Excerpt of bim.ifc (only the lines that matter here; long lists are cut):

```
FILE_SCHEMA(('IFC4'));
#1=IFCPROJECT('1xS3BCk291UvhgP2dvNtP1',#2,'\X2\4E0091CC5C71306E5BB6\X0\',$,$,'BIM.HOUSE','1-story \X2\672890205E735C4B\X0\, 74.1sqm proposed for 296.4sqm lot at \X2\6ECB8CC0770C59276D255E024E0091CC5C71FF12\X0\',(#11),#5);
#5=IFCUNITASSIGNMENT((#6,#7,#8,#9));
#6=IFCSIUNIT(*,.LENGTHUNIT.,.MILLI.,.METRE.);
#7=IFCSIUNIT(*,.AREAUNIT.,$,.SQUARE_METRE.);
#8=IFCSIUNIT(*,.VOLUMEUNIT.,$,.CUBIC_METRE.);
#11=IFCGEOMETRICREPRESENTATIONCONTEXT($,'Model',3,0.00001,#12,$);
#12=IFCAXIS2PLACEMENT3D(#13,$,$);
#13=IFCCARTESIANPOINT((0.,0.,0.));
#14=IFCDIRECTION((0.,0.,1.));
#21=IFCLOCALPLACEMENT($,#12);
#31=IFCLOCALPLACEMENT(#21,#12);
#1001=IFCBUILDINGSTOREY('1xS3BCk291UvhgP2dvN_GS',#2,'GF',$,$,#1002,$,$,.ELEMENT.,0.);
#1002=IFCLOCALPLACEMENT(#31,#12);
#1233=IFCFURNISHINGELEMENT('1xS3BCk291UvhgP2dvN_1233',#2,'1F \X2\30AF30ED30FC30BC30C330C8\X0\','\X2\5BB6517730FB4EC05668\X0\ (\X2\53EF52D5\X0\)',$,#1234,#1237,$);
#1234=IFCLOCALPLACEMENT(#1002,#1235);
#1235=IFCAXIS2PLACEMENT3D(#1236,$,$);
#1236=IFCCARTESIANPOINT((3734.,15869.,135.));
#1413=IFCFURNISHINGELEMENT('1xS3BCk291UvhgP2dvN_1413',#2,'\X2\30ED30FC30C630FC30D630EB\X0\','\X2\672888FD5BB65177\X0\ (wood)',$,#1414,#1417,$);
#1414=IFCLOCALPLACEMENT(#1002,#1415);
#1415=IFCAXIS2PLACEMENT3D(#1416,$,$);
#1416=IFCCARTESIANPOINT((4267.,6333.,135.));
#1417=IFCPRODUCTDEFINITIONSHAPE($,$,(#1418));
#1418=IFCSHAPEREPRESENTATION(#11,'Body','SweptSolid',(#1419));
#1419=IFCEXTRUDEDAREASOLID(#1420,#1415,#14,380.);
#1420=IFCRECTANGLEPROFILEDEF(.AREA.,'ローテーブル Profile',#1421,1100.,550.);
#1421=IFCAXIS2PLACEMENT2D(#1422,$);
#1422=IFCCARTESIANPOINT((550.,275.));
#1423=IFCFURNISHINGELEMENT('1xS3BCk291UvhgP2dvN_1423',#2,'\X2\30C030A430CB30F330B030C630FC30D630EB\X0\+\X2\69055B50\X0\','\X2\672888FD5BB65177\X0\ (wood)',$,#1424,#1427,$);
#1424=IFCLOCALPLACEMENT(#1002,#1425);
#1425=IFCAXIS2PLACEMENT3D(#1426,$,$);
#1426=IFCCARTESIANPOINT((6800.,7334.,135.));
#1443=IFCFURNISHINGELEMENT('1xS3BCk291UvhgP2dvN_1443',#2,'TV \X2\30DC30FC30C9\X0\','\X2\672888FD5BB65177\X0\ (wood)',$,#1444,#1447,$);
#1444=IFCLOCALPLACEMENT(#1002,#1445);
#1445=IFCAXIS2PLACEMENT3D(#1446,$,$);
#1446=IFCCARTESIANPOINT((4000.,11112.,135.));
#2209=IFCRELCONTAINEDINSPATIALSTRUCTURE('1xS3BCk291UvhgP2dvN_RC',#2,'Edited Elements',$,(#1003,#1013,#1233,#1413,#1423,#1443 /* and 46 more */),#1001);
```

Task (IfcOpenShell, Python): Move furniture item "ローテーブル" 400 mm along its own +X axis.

```python
import ifcopenshell
import ifcopenshell.api.geometry
import ifcopenshell.util.placement

model = ifcopenshell.open("bim.ifc")

item = model.by_guid("1xS3BCk291UvhgP2dvN_1413")
matrix = ifcopenshell.util.placement.get_local_placement(item.ObjectPlacement)
matrix[:3, 3] += matrix[:3, 0] * 400.0
ifcopenshell.api.geometry.edit_object_placement(model, product=item, matrix=matrix, is_si=False)

print(ifcopenshell.util.placement.get_local_placement(item.ObjectPlacement).round(3) + 0.0)

model.write("bim_v2.ifc")
```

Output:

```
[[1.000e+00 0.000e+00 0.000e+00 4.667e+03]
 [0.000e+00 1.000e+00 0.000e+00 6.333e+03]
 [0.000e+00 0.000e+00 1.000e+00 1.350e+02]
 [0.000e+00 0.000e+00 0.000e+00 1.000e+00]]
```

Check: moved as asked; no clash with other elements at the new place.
